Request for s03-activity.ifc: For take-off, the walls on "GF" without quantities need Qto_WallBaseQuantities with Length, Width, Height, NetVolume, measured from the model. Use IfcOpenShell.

First a look at what the model holds.

```python
import ifcopenshell
import ifcopenshell.util.element
import ifcopenshell.util.unit

model = ifcopenshell.open("s03-activity.ifc")
print(model.schema)
for unit_type in ("LENGTHUNIT", "AREAUNIT", "VOLUMEUNIT"):
    print(unit_type, ifcopenshell.util.unit.calculate_unit_scale(model, unit_type))
storey = next(s for s in model.by_type("IfcBuildingStorey") if s.Name == "GF")
walls = [e for e in ifcopenshell.util.element.get_decomposition(storey) if e.is_a("IfcWall")]
for e in sorted(walls, key=lambda e: e.id()):
    print(e.id(), e.is_a(), e.Name, list(ifcopenshell.util.element.get_psets(e, qtos_only=True)), sep=" | ")
```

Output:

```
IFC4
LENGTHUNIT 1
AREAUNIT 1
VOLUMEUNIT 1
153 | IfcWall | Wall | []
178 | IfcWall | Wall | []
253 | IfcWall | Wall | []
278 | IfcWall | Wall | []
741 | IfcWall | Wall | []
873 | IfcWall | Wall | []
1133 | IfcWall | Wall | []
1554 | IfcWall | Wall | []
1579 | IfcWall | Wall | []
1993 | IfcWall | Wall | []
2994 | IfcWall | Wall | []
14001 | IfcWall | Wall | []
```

```python
import ifcopenshell
import ifcopenshell.api.pset
import ifcopenshell.geom
import ifcopenshell.util.element
import ifcopenshell.util.shape
import ifcopenshell.util.unit

model = ifcopenshell.open("s03-activity.ifc")
unit_scale = ifcopenshell.util.unit.calculate_unit_scale(model)
volume_scale = ifcopenshell.util.unit.calculate_unit_scale(model, "VOLUMEUNIT")
settings = ifcopenshell.geom.settings()

storey = next(s for s in model.by_type("IfcBuildingStorey") if s.Name == "GF")
walls = [e for e in ifcopenshell.util.element.get_decomposition(storey) if e.is_a("IfcWall")]

for e in sorted(walls, key=lambda e: e.id()):
    if ifcopenshell.util.element.get_psets(e, qtos_only=True, should_inherit=False):
        continue
    # Geometry comes back in metres, in the element's own axes.
    shape = ifcopenshell.geom.create_shape(settings, e)
    values = {
        "Length": ifcopenshell.util.shape.get_x(shape.geometry) / unit_scale,
        "Width": ifcopenshell.util.shape.get_y(shape.geometry) / unit_scale,
        "Height": ifcopenshell.util.shape.get_z(shape.geometry) / unit_scale,
        "NetVolume": ifcopenshell.util.shape.get_volume(shape.geometry) / volume_scale,
    }
    qto = ifcopenshell.api.pset.add_qto(model, product=e, name="Qto_WallBaseQuantities")
    ifcopenshell.api.pset.edit_qto(model, qto=qto, properties=values)
    print(e.id(), {k: round(v, 3) for k, v in values.items()})

model.write("s03-activity_edited.ifc")
```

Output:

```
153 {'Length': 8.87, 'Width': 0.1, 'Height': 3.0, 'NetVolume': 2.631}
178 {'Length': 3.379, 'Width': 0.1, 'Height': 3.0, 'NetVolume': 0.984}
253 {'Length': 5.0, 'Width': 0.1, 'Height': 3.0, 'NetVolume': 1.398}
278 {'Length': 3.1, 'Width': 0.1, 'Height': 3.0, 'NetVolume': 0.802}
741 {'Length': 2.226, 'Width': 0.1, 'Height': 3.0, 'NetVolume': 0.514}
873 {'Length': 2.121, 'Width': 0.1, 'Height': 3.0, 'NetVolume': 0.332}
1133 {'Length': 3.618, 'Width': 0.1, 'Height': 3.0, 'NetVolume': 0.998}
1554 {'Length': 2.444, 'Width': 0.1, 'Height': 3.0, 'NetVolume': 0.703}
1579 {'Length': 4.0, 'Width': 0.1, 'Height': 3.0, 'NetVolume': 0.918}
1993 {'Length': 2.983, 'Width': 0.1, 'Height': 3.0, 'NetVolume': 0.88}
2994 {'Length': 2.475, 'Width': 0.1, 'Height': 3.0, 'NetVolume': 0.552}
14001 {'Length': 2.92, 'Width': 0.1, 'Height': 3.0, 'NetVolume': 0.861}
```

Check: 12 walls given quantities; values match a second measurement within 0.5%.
